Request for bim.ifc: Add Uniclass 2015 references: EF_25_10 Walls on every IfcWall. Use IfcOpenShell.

First a look at what the model holds.

```python
import ifcopenshell

model = ifcopenshell.open("bim.ifc")
print(model.schema)
print("classifications:", [c.Name for c in model.by_type("IfcClassification")])
for ifc_class in ("IfcDoor", "IfcRoof", "IfcStair", "IfcWall", "IfcWindow"):
    print(ifc_class, len(model.by_type(ifc_class)))
```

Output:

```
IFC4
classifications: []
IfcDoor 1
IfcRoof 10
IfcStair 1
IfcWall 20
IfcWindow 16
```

```python
import ifcopenshell
import ifcopenshell.api.classification

model = ifcopenshell.open("bim.ifc")

system = ifcopenshell.api.classification.add_classification(model, classification="Uniclass 2015")

codes = {
    "IfcWall": ("EF_25_10", "Walls"),
}
for ifc_class, (code, name) in codes.items():
    products = model.by_type(ifc_class)
    ifcopenshell.api.classification.add_reference(
        model, products=products, classification=system, identification=code, name=name
    )
    print(code, len(products))

model.write("bim-out.ifc")
```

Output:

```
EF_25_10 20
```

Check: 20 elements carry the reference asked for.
